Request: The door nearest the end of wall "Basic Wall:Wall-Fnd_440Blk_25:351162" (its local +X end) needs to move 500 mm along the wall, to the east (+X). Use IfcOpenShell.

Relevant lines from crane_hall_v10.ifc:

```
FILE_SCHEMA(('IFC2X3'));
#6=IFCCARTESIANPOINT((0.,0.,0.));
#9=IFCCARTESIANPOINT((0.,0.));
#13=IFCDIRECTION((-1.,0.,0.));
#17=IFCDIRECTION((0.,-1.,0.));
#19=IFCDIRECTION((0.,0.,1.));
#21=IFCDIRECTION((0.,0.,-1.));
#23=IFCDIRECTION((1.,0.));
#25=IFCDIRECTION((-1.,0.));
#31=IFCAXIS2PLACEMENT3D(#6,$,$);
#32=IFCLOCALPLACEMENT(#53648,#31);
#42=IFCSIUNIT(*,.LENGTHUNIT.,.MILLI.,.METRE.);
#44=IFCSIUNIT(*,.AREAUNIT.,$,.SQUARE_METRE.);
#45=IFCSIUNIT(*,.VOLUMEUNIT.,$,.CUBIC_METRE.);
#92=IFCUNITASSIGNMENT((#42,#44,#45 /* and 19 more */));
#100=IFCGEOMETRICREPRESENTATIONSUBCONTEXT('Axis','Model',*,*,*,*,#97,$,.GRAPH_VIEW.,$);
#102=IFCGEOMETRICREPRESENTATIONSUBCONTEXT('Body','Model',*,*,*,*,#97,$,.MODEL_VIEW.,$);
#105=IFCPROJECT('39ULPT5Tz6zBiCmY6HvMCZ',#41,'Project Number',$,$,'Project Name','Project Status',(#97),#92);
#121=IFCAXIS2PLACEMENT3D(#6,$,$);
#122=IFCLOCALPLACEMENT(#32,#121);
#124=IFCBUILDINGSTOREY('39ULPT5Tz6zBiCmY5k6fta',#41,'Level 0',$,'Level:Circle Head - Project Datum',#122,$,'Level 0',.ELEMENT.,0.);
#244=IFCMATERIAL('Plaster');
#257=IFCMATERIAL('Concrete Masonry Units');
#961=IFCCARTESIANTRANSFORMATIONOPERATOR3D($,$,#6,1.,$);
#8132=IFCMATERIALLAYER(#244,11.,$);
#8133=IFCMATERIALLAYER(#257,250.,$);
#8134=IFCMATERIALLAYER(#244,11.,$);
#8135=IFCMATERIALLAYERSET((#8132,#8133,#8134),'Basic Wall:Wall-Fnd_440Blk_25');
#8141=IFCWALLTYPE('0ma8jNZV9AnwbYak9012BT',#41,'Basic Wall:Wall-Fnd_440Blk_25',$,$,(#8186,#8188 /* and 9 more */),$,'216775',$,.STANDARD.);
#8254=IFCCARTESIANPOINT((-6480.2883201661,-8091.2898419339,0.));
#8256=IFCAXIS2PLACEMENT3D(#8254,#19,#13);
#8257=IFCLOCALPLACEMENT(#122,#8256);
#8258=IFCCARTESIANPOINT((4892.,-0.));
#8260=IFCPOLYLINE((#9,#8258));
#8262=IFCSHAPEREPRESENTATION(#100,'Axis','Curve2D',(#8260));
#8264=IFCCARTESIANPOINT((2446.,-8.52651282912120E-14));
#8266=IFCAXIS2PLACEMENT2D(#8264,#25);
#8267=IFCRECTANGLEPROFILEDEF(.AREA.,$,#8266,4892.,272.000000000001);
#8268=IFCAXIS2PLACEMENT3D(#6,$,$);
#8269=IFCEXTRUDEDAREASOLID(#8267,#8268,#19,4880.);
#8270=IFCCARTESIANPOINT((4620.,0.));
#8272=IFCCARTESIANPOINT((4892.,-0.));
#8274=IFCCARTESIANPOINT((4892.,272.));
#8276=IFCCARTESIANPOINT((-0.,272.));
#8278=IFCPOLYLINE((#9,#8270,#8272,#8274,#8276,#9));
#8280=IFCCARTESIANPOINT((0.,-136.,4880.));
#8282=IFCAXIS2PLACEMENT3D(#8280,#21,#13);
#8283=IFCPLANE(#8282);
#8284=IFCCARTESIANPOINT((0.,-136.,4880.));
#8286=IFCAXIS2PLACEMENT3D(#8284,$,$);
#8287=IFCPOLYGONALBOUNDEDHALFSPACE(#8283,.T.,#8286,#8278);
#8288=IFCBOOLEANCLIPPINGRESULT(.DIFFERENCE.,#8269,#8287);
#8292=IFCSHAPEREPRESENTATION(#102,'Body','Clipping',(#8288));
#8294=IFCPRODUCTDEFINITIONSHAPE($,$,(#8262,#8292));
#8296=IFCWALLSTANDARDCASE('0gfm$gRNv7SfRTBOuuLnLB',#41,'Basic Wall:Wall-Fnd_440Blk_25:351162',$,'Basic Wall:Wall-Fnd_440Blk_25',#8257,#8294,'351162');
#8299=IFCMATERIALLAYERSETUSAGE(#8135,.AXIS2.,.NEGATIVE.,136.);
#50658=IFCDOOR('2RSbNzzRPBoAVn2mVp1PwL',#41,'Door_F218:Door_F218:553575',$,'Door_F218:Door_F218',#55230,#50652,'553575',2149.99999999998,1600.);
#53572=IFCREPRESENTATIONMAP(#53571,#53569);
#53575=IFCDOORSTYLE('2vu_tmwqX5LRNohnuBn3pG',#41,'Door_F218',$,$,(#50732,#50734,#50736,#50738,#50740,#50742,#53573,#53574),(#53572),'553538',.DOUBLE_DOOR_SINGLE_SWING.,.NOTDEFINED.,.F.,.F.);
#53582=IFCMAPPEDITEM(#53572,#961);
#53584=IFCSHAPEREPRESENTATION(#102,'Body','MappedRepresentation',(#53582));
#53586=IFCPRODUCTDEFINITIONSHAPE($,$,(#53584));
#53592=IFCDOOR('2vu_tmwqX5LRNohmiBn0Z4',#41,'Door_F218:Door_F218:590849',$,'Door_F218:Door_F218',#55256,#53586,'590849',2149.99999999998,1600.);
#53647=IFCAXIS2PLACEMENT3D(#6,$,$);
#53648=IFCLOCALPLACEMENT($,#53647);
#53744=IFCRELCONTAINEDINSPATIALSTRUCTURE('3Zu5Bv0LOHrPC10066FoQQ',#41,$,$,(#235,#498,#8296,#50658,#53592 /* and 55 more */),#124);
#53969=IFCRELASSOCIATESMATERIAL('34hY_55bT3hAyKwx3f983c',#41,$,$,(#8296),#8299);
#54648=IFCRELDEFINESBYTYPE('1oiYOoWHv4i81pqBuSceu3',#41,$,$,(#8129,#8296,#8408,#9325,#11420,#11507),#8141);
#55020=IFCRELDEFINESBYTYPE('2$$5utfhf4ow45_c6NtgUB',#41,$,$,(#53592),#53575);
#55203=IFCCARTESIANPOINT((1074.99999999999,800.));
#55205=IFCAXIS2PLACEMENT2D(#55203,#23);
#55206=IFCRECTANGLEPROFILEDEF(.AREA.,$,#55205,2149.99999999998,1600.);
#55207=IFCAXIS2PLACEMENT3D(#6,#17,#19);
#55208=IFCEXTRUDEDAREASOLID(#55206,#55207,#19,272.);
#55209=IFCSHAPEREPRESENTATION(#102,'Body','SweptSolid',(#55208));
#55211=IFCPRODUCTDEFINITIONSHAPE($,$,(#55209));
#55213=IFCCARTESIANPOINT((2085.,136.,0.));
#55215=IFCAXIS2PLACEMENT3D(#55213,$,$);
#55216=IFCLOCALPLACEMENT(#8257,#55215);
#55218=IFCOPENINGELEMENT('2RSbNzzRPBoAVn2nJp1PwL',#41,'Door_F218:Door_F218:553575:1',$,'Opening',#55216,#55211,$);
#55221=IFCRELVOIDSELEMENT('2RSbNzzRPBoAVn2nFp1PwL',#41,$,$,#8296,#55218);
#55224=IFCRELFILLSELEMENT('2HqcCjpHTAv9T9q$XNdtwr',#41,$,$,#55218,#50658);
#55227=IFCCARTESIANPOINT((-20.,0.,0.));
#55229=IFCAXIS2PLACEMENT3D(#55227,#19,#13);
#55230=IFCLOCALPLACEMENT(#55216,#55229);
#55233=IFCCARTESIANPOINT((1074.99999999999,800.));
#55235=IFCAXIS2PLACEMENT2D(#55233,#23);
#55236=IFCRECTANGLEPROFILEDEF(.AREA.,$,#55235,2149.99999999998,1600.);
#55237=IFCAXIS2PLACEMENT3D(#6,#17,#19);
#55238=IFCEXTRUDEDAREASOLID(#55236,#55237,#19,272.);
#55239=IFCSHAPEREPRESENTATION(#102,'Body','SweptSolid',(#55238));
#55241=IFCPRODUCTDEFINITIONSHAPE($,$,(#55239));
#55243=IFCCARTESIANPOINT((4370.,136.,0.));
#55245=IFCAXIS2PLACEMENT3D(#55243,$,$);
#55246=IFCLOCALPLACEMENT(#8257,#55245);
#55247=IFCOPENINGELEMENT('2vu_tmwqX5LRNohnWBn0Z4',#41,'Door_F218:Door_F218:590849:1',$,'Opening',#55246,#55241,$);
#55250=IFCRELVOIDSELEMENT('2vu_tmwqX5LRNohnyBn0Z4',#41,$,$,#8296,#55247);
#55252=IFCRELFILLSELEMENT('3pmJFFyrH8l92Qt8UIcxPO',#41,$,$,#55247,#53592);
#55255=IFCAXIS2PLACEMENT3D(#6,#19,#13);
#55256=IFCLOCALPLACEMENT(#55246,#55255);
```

```python
import ifcopenshell
import ifcopenshell.api.geometry
import ifcopenshell.util.placement
import ifcopenshell.util.unit

model = ifcopenshell.open("crane_hall_v10.ifc")
unit_scale = ifcopenshell.util.unit.calculate_unit_scale(model)

door = model.by_guid("2vu_tmwqX5LRNohmiBn0Z4")
opening = door.FillsVoids[0].RelatingOpeningElement
wall = opening.VoidsElements[0].RelatingBuildingElement

wall_matrix = ifcopenshell.util.placement.get_local_placement(wall.ObjectPlacement)
shift = wall_matrix[:3, 0] * -0.5 / unit_scale
before = ifcopenshell.util.placement.get_local_placement(door.ObjectPlacement)[:3, 3].copy()

# The door is placed relative to its opening, so it follows when the opening moves.
matrix = ifcopenshell.util.placement.get_local_placement(opening.ObjectPlacement)
matrix[:3, 3] += shift
ifcopenshell.api.geometry.edit_object_placement(
    model, product=opening, matrix=matrix, is_si=False, should_transform_children=True
)

after = ifcopenshell.util.placement.get_local_placement(door.ObjectPlacement)[:3, 3]
print("door moved by", (after - before).round(3) + 0.0)

model.write("crane_hall_v10_edited.ifc")
```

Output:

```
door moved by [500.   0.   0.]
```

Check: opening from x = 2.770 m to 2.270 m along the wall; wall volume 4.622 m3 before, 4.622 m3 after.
